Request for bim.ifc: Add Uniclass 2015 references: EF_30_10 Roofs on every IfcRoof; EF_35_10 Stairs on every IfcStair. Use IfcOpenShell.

First a look at what the model holds.

```python
import ifcopenshell

model = ifcopenshell.open("bim.ifc")
print(model.schema)
print("classifications:", [c.Name for c in model.by_type("IfcClassification")])
for ifc_class in ("IfcDoor", "IfcRoof", "IfcStair", "IfcWall", "IfcWindow"):
    print(ifc_class, len(model.by_type(ifc_class)))
```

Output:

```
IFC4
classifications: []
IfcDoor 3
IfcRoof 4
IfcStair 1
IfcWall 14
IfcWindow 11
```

```python
import ifcopenshell
import ifcopenshell.api.classification

model = ifcopenshell.open("bim.ifc")

system = ifcopenshell.api.classification.add_classification(model, classification="Uniclass 2015")

codes = {
    "IfcRoof": ("EF_30_10", "Roofs"),
    "IfcStair": ("EF_35_10", "Stairs"),
}
for ifc_class, (code, name) in codes.items():
    products = model.by_type(ifc_class)
    ifcopenshell.api.classification.add_reference(
        model, products=products, classification=system, identification=code, name=name
    )
    print(code, len(products))

model.write("bim_v2.ifc")
```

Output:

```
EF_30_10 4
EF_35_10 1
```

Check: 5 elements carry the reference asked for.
